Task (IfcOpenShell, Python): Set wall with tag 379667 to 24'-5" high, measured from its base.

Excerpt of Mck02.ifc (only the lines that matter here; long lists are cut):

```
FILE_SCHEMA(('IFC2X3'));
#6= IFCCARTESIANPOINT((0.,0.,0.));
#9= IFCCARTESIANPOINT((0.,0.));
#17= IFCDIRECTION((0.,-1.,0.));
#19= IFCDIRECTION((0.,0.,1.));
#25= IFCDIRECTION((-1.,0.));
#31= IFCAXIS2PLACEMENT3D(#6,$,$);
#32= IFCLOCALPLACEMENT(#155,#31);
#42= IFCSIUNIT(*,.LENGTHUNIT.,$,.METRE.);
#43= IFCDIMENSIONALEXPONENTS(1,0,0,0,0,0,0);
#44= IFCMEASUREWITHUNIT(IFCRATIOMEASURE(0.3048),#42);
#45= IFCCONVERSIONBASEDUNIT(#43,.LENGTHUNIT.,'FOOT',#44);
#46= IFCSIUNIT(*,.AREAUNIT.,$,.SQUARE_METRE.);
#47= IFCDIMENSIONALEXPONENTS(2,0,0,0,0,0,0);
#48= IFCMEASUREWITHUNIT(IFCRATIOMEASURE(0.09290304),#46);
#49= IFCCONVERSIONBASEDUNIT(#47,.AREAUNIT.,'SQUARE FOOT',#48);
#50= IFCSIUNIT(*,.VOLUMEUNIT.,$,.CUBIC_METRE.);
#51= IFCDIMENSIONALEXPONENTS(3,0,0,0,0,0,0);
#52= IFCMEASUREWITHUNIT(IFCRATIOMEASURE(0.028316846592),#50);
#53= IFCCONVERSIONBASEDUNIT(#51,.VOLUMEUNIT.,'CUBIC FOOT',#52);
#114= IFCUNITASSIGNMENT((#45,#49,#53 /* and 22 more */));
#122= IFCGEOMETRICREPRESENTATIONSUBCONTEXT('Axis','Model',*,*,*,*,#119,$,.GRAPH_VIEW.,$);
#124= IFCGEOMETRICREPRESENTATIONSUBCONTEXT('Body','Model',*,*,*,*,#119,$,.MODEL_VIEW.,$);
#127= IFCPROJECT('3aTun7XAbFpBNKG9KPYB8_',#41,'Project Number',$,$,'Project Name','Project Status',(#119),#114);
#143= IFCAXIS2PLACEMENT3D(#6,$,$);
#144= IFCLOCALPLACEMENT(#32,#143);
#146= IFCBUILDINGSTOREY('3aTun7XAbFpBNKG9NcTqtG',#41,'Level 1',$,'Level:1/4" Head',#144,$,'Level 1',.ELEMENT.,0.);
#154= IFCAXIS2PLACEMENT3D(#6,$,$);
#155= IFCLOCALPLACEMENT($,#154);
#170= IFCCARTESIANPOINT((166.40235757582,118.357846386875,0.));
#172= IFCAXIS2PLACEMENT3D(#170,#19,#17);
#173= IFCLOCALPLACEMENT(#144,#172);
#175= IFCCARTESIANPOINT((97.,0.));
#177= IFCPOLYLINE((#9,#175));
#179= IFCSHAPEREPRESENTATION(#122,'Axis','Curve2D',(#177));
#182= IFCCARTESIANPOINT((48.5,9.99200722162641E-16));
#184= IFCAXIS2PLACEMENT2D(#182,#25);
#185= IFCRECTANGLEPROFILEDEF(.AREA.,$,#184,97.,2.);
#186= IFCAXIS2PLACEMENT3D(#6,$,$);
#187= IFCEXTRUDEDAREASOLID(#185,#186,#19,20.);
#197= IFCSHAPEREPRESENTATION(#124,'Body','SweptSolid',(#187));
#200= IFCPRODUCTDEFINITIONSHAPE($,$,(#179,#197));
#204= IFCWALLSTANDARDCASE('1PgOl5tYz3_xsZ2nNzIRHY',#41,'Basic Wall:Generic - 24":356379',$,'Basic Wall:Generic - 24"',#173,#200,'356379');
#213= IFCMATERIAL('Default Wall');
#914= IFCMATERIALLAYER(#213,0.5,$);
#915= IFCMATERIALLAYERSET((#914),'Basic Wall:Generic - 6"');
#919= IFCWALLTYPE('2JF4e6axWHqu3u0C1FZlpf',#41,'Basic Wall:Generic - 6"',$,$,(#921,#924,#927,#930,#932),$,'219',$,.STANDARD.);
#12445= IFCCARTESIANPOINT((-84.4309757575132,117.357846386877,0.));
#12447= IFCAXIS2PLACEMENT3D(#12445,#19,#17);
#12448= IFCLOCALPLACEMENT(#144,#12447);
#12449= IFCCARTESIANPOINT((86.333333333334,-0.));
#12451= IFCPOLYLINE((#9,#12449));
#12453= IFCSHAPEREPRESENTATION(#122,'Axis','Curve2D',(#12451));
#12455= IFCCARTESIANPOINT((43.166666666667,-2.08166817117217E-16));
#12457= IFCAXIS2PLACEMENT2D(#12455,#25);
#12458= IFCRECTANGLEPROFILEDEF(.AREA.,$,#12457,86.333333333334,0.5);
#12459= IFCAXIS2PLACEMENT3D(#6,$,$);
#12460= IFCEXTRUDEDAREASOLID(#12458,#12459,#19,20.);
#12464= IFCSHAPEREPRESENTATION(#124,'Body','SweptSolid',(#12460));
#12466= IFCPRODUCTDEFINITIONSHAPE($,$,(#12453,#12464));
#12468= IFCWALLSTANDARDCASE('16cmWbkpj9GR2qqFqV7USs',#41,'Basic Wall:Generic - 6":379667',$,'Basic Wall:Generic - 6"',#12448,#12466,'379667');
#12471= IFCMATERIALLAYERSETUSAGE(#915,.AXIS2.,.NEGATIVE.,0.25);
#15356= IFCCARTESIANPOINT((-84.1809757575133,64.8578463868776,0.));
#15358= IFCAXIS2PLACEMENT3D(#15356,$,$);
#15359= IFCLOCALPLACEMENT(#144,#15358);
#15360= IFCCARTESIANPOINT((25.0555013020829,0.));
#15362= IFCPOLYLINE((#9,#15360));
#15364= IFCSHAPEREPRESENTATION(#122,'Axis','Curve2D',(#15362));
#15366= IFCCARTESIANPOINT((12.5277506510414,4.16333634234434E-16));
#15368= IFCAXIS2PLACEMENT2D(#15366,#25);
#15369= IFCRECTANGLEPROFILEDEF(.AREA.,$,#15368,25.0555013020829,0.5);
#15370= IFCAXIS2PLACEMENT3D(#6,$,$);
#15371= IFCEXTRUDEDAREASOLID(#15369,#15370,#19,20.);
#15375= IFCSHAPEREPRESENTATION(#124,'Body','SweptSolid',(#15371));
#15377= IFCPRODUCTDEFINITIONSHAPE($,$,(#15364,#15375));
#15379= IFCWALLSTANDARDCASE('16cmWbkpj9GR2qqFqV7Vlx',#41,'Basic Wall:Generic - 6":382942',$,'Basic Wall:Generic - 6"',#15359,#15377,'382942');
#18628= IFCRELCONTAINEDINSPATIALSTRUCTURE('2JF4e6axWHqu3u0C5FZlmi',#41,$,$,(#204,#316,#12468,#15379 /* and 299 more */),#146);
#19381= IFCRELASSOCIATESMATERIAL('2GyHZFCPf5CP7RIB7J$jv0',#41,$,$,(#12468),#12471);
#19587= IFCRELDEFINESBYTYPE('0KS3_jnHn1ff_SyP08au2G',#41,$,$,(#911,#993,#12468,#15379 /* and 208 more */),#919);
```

```python
import ifcopenshell
import ifcopenshell.geom
import ifcopenshell.util.representation
import ifcopenshell.util.shape
import ifcopenshell.util.unit

model = ifcopenshell.open("Mck02.ifc")
unit_scale = ifcopenshell.util.unit.calculate_unit_scale(model)
settings = ifcopenshell.geom.settings()


def volume(element):
    """Net volume in cubic metres, openings subtracted."""
    shape = ifcopenshell.geom.create_shape(settings, element)
    return ifcopenshell.util.shape.get_volume(shape.geometry)


wall = model.by_guid("16cmWbkpj9GR2qqFqV7USs")
before = volume(wall)

body = ifcopenshell.util.representation.get_representation(wall, "Model", "Body")
solid = body.Items[0]
old_height = solid.Depth
solid.Depth = 293 * 0.0254 / unit_scale
after = volume(wall)

print(f"height {old_height:g} -> {solid.Depth:g}, volume {before:.3f} -> {after:.3f} m3")

model.write("Mck02_v2.ifc")
```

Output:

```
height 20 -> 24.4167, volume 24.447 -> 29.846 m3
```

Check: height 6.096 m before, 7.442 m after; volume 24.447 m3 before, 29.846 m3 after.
